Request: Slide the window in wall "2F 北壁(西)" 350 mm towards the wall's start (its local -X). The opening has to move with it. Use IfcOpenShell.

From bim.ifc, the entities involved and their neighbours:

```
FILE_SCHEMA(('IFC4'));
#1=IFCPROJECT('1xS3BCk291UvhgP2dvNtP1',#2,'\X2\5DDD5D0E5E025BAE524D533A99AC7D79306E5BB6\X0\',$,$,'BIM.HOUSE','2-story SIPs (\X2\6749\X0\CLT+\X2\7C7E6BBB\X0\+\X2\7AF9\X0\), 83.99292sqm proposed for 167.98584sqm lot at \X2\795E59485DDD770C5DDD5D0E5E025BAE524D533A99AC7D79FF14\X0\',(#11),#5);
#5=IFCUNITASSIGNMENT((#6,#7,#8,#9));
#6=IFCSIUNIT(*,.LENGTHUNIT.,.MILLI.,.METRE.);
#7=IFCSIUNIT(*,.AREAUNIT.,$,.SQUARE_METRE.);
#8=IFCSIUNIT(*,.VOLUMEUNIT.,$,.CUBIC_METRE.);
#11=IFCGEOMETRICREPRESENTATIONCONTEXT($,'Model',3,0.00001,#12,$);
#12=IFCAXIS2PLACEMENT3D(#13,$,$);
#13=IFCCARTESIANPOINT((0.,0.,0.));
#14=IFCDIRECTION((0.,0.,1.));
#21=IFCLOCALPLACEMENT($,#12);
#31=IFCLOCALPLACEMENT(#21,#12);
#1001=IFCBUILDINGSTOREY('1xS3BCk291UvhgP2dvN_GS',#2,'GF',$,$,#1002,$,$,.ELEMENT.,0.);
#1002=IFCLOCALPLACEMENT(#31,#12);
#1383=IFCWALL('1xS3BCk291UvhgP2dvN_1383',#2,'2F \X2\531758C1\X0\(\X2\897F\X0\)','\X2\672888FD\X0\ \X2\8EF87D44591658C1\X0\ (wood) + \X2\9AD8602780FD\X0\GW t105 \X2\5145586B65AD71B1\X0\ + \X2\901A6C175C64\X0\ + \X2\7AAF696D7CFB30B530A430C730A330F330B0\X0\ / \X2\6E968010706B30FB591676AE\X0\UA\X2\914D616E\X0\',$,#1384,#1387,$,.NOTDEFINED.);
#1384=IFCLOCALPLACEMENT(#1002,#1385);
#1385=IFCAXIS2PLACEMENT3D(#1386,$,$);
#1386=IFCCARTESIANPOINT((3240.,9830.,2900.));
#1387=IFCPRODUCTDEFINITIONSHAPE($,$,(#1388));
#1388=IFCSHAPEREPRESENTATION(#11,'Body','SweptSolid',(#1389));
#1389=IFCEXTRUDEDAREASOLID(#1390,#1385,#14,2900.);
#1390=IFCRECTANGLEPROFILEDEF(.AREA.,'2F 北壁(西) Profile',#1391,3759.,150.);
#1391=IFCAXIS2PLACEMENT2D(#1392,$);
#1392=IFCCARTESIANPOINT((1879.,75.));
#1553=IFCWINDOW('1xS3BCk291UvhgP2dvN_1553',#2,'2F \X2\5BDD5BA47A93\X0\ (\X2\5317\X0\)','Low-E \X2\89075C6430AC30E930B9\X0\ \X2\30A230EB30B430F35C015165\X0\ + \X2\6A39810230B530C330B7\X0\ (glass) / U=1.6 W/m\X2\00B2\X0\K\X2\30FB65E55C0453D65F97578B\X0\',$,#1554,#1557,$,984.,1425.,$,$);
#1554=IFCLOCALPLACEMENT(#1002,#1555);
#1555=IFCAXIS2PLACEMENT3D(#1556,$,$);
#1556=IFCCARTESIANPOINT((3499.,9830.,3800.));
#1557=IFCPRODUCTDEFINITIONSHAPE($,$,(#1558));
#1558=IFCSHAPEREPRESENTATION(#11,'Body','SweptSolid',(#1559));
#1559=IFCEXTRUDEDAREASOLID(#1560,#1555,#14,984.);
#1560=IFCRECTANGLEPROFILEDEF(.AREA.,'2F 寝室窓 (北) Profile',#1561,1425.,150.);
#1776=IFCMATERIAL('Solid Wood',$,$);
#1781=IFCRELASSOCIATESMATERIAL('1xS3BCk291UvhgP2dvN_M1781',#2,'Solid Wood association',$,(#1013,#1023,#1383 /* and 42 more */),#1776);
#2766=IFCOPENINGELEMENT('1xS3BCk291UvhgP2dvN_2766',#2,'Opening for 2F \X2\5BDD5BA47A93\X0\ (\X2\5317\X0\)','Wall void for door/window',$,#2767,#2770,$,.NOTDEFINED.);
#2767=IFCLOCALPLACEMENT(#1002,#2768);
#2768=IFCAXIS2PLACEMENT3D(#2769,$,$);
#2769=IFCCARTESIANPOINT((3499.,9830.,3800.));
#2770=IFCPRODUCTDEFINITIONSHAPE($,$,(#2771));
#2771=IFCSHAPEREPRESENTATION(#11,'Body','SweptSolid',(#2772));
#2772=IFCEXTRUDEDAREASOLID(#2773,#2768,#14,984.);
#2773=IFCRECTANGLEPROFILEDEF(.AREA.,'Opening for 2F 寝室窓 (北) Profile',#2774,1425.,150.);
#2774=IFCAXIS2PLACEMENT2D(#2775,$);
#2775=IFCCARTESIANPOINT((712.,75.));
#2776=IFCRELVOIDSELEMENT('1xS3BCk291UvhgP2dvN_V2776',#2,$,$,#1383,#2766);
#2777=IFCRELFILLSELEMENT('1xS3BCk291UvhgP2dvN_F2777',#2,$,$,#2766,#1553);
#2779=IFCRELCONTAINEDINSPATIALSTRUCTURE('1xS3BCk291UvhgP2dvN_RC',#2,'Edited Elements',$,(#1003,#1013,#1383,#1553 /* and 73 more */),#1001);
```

```python
import ifcopenshell
import ifcopenshell.api.geometry
import ifcopenshell.util.placement
import ifcopenshell.util.unit

model = ifcopenshell.open("bim.ifc")
unit_scale = ifcopenshell.util.unit.calculate_unit_scale(model)

window = model.by_id(1553)
opening = window.FillsVoids[0].RelatingOpeningElement
wall = opening.VoidsElements[0].RelatingBuildingElement

wall_matrix = ifcopenshell.util.placement.get_local_placement(wall.ObjectPlacement)
shift = wall_matrix[:3, 0] * -0.35 / unit_scale
before = ifcopenshell.util.placement.get_local_placement(window.ObjectPlacement)[:3, 3].copy()

# The window is not placed relative to its opening, so move both.
for product in (opening, window):
    matrix = ifcopenshell.util.placement.get_local_placement(product.ObjectPlacement)
    matrix[:3, 3] += shift
    ifcopenshell.api.geometry.edit_object_placement(model, product=product, matrix=matrix, is_si=False)

after = ifcopenshell.util.placement.get_local_placement(window.ObjectPlacement)[:3, 3]
print("window moved by", (after - before).round(3) + 0.0)

model.write("bim_edited.ifc")
```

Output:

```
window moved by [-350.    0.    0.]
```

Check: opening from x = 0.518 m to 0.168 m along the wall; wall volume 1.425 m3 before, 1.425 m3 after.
